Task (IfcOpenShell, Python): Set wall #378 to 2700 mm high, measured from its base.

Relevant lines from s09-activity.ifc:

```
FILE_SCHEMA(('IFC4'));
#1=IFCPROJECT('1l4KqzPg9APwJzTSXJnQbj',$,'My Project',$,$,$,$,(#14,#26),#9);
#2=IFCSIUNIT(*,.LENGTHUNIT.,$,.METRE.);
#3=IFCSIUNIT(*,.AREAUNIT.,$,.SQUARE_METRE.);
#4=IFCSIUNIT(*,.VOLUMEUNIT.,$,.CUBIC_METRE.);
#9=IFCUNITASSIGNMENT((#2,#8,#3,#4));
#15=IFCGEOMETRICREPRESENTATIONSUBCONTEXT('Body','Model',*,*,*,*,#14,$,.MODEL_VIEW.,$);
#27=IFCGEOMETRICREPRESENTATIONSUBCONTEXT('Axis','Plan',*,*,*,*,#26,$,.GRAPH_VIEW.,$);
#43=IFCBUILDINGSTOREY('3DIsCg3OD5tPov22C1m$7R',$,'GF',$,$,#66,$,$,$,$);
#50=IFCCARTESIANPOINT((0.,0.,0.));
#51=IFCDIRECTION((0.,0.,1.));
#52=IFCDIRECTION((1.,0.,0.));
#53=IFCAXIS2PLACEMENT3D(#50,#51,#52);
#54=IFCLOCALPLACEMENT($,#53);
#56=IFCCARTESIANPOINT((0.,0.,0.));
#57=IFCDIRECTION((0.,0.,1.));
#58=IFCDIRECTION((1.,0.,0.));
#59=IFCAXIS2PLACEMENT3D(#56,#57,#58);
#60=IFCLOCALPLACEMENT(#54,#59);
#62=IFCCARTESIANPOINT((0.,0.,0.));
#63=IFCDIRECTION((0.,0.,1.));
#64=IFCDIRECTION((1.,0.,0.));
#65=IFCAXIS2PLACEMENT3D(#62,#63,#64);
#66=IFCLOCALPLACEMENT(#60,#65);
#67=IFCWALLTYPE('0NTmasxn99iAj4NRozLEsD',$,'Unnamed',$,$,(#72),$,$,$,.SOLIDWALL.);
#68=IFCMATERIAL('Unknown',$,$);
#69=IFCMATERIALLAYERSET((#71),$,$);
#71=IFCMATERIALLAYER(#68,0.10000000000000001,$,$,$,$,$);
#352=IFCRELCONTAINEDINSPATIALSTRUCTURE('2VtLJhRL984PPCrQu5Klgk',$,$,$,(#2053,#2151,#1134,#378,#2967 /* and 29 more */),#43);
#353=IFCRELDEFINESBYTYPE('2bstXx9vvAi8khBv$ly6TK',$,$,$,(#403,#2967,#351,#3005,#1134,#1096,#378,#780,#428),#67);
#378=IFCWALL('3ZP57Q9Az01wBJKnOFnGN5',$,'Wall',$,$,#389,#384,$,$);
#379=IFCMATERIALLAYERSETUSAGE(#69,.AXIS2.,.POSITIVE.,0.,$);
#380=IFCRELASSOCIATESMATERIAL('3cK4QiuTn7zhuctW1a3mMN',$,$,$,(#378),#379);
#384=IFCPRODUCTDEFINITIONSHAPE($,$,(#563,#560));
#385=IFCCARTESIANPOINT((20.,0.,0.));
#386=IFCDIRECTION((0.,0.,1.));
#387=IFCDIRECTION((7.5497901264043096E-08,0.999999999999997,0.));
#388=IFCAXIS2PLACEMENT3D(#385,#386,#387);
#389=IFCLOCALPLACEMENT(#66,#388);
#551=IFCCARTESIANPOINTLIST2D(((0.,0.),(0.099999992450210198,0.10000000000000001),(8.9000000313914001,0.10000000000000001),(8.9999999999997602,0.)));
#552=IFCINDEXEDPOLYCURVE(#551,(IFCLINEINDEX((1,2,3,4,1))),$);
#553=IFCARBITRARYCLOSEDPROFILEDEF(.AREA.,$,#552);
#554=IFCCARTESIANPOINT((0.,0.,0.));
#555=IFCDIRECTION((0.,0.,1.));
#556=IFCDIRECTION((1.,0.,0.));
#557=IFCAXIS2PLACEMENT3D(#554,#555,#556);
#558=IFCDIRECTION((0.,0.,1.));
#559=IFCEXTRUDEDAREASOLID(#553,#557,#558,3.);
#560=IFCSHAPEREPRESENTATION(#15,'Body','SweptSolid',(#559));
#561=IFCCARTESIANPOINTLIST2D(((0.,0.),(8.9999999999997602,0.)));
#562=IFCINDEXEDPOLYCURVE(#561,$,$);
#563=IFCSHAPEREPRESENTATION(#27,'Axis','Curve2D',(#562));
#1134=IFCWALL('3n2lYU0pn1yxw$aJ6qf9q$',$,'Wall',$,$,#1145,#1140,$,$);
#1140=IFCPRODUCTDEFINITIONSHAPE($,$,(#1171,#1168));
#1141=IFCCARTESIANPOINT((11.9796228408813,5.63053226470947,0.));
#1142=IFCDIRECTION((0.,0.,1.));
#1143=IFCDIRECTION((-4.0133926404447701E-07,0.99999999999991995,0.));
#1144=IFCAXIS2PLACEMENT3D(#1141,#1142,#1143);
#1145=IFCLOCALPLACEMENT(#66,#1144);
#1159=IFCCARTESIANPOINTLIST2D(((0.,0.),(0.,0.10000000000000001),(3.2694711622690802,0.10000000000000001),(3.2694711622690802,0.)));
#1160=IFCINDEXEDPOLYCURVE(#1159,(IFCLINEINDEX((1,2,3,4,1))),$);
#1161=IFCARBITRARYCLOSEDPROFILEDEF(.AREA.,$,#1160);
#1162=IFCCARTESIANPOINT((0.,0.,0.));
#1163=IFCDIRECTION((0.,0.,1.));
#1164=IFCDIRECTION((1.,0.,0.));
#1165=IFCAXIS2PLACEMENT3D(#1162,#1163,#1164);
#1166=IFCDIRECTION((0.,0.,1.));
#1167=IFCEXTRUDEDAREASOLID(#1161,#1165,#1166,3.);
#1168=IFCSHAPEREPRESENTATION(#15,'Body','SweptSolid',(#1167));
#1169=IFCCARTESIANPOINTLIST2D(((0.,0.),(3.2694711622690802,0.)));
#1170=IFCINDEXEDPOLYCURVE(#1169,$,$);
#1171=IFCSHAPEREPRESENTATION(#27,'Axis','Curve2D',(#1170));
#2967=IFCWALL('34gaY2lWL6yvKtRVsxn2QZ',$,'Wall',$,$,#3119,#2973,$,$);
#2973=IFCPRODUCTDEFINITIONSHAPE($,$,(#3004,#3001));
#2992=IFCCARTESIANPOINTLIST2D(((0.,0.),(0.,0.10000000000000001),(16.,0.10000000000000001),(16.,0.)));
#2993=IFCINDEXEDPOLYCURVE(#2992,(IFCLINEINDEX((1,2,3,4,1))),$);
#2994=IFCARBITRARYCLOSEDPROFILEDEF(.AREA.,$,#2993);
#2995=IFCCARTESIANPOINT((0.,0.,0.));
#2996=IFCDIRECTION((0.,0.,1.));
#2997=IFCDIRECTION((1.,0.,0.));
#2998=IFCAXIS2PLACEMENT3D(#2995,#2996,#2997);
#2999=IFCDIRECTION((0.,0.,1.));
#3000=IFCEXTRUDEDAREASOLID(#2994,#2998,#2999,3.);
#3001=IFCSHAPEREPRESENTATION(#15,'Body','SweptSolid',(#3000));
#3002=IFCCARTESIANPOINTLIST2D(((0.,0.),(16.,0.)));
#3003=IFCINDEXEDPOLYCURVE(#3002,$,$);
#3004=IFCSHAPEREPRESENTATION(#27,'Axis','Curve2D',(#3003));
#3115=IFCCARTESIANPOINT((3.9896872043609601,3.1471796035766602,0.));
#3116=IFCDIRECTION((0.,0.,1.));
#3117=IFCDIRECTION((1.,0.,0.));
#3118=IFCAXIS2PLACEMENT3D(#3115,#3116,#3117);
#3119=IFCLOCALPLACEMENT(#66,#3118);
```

```python
import ifcopenshell
import ifcopenshell.geom
import ifcopenshell.util.representation
import ifcopenshell.util.shape

model = ifcopenshell.open("s09-activity.ifc")
settings = ifcopenshell.geom.settings()


def volume(element):
    """Net volume in cubic metres, openings subtracted."""
    shape = ifcopenshell.geom.create_shape(settings, element)
    return ifcopenshell.util.shape.get_volume(shape.geometry)


wall = model.by_guid("3ZP57Q9Az01wBJKnOFnGN5")
before = volume(wall)

body = ifcopenshell.util.representation.get_representation(wall, "Model", "Body")
solid = body.Items[0]
old_height = solid.Depth
solid.Depth = 2.7
after = volume(wall)

print(f"height {old_height:g} -> {solid.Depth:g}, volume {before:.3f} -> {after:.3f} m3")

model.write("s09-activity_rev.ifc")
```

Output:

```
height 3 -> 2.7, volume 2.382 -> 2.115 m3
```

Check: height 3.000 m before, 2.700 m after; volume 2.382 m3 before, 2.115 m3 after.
